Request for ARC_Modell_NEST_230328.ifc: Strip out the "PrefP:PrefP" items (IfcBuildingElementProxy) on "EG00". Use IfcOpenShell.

First a look at what the model holds.

```python
import ifcopenshell
import ifcopenshell.util.element

model = ifcopenshell.open("ARC_Modell_NEST_230328.ifc")
print(model.schema)
storey = next(s for s in model.by_type("IfcBuildingStorey") if s.Name == "EG00")
proxies = [e for e in ifcopenshell.util.element.get_decomposition(storey) if e.is_a("IfcBuildingElementProxy")]
seen = {}
for e in proxies:
    element_type = ifcopenshell.util.element.get_type(e)
    name = element_type.Name if element_type not in (None, e) else None
    seen[name] = seen.get(name, 0) + 1
for name, count in sorted(seen.items(), key=str):
    print(count, "x", name)
```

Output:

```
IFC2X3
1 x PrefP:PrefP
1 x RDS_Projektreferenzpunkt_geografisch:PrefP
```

```python
import ifcopenshell
import ifcopenshell.api.root
import ifcopenshell.util.element

model = ifcopenshell.open("ARC_Modell_NEST_230328.ifc")

storey = next(s for s in model.by_type("IfcBuildingStorey") if s.Name == "EG00")
proxies = [e for e in ifcopenshell.util.element.get_decomposition(storey) if e.is_a("IfcBuildingElementProxy")]
targets = [e for e in proxies if (t := ifcopenshell.util.element.get_type(e)) not in (None, e) and t.Name == "PrefP:PrefP"]

for e in targets:
    ifcopenshell.api.root.remove_product(model, product=e)
print(len(targets), "removed")

model.write("ARC_Modell_NEST_230328_edited.ifc")
```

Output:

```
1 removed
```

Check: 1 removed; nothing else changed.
